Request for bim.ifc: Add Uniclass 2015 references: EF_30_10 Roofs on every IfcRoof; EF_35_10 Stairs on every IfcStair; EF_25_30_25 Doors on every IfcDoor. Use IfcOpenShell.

First a look at what the model holds.

```python
import ifcopenshell

model = ifcopenshell.open("bim.ifc")
print(model.schema)
print("classifications:", [c.Name for c in model.by_type("IfcClassification")])
for ifc_class in ("IfcDoor", "IfcRoof", "IfcStair", "IfcWall", "IfcWindow"):
    print(ifc_class, len(model.by_type(ifc_class)))
```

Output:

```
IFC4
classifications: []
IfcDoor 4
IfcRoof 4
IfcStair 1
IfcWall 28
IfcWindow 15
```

```python
import ifcopenshell
import ifcopenshell.api.classification

model = ifcopenshell.open("bim.ifc")

system = ifcopenshell.api.classification.add_classification(model, classification="Uniclass 2015")

codes = {
    "IfcRoof": ("EF_30_10", "Roofs"),
    "IfcStair": ("EF_35_10", "Stairs"),
    "IfcDoor": ("EF_25_30_25", "Doors"),
}
for ifc_class, (code, name) in codes.items():
    products = model.by_type(ifc_class)
    ifcopenshell.api.classification.add_reference(
        model, products=products, classification=system, identification=code, name=name
    )
    print(code, len(products))

model.write("bim_edited.ifc")
```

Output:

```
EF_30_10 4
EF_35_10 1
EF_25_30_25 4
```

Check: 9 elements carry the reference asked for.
